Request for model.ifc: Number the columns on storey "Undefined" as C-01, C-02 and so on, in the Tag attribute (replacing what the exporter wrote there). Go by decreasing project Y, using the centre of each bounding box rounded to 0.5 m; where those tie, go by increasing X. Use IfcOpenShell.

First a look at what the model holds.

```python
import ifcopenshell
import ifcopenshell.util.element
import ifcopenshell.util.placement

model = ifcopenshell.open("model.ifc")
print(model.schema)
storey = next(s for s in model.by_type("IfcBuildingStorey") if s.Name == "Undefined")
columns = [e for e in ifcopenshell.util.element.get_decomposition(storey) if e.is_a("IfcColumn")]
for e in sorted(columns, key=lambda e: e.id()):
    origin = ifcopenshell.util.placement.get_local_placement(e.ObjectPlacement)[:3, 3]
    print(e.id(), e.Tag, e.Name, origin.round(2) + 0.0, sep=" | ")
```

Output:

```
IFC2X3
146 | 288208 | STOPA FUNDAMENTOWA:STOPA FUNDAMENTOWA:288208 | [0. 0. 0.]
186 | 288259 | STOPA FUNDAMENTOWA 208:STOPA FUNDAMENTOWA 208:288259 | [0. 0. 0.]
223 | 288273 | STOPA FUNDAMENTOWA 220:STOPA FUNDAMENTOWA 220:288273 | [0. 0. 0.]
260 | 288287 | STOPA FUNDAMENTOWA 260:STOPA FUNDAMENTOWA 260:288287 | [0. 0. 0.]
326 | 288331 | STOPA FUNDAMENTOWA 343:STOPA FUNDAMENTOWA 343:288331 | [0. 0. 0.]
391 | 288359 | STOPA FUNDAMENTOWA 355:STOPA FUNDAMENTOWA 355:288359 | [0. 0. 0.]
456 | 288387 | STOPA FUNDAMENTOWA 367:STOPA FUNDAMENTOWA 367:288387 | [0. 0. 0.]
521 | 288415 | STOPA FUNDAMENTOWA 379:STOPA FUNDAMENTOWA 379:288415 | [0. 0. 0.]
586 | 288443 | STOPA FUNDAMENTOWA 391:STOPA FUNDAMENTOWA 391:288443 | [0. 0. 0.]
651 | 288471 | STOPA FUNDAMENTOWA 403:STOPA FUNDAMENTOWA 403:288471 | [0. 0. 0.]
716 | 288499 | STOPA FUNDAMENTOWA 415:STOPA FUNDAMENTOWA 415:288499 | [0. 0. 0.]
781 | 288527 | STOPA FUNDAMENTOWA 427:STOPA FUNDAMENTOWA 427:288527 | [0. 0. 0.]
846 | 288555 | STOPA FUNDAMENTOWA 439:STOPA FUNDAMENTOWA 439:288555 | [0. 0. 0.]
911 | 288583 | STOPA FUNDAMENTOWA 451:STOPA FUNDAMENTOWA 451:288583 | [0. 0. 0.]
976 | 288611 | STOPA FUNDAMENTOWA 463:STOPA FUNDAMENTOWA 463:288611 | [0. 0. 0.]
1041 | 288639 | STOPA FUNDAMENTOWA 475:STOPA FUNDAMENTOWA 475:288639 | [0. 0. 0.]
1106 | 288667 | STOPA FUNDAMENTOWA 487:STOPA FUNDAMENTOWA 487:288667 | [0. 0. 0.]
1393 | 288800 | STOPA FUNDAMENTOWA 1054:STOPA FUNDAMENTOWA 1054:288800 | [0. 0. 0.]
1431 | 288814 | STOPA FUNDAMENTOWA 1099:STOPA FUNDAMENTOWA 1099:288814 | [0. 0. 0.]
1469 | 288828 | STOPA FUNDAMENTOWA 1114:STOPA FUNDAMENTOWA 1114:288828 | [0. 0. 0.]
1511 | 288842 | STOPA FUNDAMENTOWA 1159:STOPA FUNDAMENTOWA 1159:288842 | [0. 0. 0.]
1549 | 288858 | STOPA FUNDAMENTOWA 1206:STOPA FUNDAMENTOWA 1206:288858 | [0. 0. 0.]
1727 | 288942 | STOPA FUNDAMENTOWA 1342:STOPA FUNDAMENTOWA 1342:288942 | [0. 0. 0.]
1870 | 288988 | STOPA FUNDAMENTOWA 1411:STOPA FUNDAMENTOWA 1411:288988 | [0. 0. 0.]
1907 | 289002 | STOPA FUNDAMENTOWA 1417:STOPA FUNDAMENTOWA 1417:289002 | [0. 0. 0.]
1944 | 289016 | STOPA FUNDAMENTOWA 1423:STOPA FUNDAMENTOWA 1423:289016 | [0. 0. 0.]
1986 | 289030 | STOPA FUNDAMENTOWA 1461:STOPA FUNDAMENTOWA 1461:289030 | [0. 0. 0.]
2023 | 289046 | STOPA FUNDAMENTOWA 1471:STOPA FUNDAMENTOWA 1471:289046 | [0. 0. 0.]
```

```python
import ifcopenshell
import ifcopenshell.geom
import ifcopenshell.util.element
import ifcopenshell.util.shape

model = ifcopenshell.open("model.ifc")
settings = ifcopenshell.geom.settings()
settings.set("use-world-coords", True)


def centre(element):
    shape = ifcopenshell.geom.create_shape(settings, element)
    return ifcopenshell.util.shape.get_bbox_centroid(shape.geometry)


storey = next(s for s in model.by_type("IfcBuildingStorey") if s.Name == "Undefined")
columns = [e for e in ifcopenshell.util.element.get_decomposition(storey) if e.is_a("IfcColumn")]

# Insertion points can sit at a corner or the storey origin, so sort by the geometry (in metres).
centres = {e: centre(e) for e in columns}
columns.sort(key=lambda e: (-round(centres[e][1] / 0.5), centres[e][0]))

for i, e in enumerate(columns, start=1):
    number = f"C-{i:02d}"
    e.Tag = number
    print(e.id(), number)

model.write("model-out.ifc")
```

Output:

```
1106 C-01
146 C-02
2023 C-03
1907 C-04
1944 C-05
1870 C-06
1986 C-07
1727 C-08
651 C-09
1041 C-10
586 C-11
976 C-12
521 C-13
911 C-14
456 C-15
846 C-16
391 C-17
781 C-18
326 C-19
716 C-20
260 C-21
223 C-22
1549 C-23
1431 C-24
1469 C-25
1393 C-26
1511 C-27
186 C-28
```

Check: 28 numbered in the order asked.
